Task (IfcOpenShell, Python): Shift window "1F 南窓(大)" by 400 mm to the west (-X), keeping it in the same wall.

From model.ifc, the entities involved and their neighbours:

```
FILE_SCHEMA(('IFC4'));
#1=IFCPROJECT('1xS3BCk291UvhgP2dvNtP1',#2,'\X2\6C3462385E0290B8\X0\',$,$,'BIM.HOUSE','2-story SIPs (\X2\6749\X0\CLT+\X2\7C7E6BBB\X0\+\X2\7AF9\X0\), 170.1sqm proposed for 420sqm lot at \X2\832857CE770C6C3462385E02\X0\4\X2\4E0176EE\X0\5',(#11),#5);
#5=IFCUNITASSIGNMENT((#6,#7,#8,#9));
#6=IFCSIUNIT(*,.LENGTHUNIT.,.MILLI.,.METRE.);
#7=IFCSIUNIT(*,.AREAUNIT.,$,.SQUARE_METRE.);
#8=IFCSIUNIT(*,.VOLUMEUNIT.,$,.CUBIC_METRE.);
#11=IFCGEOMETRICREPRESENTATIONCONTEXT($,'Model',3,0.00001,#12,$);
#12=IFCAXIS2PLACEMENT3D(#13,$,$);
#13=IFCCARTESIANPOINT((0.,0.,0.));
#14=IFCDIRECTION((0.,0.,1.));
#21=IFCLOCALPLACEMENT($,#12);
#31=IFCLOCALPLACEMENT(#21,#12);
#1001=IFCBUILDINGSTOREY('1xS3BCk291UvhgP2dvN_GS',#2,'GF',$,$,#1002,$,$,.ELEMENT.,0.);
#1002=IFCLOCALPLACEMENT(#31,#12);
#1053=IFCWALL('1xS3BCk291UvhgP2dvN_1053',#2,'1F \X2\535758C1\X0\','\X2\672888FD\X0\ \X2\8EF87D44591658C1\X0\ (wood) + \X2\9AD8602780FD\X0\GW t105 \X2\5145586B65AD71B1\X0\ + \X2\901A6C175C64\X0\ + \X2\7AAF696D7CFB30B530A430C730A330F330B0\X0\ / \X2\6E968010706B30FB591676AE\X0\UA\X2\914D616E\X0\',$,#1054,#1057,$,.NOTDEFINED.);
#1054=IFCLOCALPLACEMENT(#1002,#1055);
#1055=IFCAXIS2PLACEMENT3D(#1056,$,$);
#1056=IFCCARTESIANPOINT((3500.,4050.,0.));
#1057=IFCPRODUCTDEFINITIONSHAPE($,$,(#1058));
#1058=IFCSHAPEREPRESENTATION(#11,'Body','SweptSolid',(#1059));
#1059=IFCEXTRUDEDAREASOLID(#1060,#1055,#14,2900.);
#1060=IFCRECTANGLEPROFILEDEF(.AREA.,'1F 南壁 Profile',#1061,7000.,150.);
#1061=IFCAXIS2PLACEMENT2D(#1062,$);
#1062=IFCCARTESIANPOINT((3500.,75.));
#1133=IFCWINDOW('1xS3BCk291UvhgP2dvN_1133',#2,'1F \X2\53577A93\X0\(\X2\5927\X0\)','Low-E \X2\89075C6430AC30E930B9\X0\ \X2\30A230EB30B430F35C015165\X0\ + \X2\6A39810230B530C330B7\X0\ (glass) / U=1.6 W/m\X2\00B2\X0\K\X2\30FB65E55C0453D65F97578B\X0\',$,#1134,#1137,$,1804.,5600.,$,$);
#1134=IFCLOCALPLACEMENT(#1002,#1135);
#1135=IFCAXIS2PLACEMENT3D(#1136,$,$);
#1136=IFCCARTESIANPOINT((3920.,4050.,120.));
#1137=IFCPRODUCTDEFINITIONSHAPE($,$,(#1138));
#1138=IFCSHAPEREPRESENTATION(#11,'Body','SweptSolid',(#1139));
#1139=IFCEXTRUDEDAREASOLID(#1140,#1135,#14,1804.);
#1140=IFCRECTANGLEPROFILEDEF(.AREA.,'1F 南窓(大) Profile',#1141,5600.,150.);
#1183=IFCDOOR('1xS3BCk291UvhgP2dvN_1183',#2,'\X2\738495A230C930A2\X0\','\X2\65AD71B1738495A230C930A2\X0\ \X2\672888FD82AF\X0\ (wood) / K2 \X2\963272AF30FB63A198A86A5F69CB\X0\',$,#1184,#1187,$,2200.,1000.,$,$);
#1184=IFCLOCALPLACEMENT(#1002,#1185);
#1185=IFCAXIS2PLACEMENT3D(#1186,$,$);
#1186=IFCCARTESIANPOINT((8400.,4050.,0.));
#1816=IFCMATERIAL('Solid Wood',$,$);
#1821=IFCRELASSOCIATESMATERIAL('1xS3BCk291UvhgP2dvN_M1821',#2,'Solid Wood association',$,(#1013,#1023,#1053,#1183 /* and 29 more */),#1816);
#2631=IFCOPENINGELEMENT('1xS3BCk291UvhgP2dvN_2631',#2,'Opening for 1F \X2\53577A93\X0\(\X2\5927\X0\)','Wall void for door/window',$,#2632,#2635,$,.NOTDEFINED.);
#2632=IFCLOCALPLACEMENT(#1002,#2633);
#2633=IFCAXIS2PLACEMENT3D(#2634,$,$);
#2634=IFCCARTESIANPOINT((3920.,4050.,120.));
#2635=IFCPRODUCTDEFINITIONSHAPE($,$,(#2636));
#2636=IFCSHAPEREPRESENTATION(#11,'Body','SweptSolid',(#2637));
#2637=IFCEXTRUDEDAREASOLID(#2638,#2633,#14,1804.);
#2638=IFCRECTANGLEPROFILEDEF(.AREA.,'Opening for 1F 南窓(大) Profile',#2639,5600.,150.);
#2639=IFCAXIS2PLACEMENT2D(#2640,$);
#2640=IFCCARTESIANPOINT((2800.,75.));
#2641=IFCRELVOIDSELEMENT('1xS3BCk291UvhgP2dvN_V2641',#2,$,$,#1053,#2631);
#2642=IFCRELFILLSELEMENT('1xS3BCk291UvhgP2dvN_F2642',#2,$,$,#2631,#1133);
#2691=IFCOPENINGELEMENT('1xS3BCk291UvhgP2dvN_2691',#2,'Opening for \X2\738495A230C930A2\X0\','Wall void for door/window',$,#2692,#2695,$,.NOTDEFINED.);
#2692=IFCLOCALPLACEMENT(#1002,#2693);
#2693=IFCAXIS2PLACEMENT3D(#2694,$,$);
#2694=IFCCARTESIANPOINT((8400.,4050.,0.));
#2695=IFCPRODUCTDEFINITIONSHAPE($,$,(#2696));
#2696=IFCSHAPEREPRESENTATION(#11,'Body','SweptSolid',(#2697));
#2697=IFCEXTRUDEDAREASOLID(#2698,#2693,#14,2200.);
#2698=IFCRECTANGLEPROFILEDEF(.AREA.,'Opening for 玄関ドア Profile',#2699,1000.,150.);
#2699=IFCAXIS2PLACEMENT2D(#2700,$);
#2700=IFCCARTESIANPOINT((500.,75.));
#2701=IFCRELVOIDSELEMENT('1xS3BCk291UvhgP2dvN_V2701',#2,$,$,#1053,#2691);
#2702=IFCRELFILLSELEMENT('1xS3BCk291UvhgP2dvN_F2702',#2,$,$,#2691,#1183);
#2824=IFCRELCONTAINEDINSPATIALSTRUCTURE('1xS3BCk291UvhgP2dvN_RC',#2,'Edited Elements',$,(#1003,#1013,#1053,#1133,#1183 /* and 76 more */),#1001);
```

```python
import ifcopenshell
import ifcopenshell.api.geometry
import ifcopenshell.util.placement

model = ifcopenshell.open("model.ifc")

window = model.by_guid("1xS3BCk291UvhgP2dvN_1133")
opening = window.FillsVoids[0].RelatingOpeningElement
wall = opening.VoidsElements[0].RelatingBuildingElement

wall_matrix = ifcopenshell.util.placement.get_local_placement(wall.ObjectPlacement)
shift = wall_matrix[:3, 0] * -400.0
before = ifcopenshell.util.placement.get_local_placement(window.ObjectPlacement)[:3, 3].copy()

# The window is not placed relative to its opening, so move both.
for product in (opening, window):
    matrix = ifcopenshell.util.placement.get_local_placement(product.ObjectPlacement)
    matrix[:3, 3] += shift
    ifcopenshell.api.geometry.edit_object_placement(model, product=product, matrix=matrix, is_si=False)

after = ifcopenshell.util.placement.get_local_placement(window.ObjectPlacement)[:3, 3]
print("window moved by", (after - before).round(3) + 0.0)

model.write("model-out.ifc")
```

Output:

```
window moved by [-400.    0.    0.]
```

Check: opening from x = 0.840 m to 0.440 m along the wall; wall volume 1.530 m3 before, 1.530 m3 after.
